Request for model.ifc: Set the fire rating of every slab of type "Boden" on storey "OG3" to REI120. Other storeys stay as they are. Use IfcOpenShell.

First a look at what the model holds.

```python
import ifcopenshell
import ifcopenshell.util.element

model = ifcopenshell.open("model.ifc")
print(model.schema)
storey = next(s for s in model.by_type("IfcBuildingStorey") if s.Name == "OG3")
slabs = [e for e in ifcopenshell.util.element.get_decomposition(storey) if e.is_a("IfcSlab")]
seen = {}
for e in slabs:
    element_type = ifcopenshell.util.element.get_type(e)
    key = (element_type.Name if element_type != e and element_type else None, ifcopenshell.util.element.get_pset(e, "Pset_SlabCommon", "FireRating"))
    seen[key] = seen.get(key, 0) + 1
for (name, value), count in sorted(seen.items(), key=str):
    print(count, "x", name, "|", value)
```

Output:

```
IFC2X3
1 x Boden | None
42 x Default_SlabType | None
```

```python
import ifcopenshell
import ifcopenshell.api.pset
import ifcopenshell.util.element

model = ifcopenshell.open("model.ifc")

storey = next(s for s in model.by_type("IfcBuildingStorey") if s.Name == "OG3")
slabs = [e for e in ifcopenshell.util.element.get_decomposition(storey) if e.is_a("IfcSlab")]

count = 0
for e in slabs:
    element_type = ifcopenshell.util.element.get_type(e)
    if element_type in (None, e) or element_type.Name != "Boden":
        continue
    # add_pset returns the element's existing set when there is one.
    pset = ifcopenshell.api.pset.add_pset(model, product=e, name="Pset_SlabCommon")
    ifcopenshell.api.pset.edit_pset(model, pset=pset, properties={"FireRating": "REI120"})
    count += 1

print(count, "slabs updated")

model.write("model_rev.ifc")
```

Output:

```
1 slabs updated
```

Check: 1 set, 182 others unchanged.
